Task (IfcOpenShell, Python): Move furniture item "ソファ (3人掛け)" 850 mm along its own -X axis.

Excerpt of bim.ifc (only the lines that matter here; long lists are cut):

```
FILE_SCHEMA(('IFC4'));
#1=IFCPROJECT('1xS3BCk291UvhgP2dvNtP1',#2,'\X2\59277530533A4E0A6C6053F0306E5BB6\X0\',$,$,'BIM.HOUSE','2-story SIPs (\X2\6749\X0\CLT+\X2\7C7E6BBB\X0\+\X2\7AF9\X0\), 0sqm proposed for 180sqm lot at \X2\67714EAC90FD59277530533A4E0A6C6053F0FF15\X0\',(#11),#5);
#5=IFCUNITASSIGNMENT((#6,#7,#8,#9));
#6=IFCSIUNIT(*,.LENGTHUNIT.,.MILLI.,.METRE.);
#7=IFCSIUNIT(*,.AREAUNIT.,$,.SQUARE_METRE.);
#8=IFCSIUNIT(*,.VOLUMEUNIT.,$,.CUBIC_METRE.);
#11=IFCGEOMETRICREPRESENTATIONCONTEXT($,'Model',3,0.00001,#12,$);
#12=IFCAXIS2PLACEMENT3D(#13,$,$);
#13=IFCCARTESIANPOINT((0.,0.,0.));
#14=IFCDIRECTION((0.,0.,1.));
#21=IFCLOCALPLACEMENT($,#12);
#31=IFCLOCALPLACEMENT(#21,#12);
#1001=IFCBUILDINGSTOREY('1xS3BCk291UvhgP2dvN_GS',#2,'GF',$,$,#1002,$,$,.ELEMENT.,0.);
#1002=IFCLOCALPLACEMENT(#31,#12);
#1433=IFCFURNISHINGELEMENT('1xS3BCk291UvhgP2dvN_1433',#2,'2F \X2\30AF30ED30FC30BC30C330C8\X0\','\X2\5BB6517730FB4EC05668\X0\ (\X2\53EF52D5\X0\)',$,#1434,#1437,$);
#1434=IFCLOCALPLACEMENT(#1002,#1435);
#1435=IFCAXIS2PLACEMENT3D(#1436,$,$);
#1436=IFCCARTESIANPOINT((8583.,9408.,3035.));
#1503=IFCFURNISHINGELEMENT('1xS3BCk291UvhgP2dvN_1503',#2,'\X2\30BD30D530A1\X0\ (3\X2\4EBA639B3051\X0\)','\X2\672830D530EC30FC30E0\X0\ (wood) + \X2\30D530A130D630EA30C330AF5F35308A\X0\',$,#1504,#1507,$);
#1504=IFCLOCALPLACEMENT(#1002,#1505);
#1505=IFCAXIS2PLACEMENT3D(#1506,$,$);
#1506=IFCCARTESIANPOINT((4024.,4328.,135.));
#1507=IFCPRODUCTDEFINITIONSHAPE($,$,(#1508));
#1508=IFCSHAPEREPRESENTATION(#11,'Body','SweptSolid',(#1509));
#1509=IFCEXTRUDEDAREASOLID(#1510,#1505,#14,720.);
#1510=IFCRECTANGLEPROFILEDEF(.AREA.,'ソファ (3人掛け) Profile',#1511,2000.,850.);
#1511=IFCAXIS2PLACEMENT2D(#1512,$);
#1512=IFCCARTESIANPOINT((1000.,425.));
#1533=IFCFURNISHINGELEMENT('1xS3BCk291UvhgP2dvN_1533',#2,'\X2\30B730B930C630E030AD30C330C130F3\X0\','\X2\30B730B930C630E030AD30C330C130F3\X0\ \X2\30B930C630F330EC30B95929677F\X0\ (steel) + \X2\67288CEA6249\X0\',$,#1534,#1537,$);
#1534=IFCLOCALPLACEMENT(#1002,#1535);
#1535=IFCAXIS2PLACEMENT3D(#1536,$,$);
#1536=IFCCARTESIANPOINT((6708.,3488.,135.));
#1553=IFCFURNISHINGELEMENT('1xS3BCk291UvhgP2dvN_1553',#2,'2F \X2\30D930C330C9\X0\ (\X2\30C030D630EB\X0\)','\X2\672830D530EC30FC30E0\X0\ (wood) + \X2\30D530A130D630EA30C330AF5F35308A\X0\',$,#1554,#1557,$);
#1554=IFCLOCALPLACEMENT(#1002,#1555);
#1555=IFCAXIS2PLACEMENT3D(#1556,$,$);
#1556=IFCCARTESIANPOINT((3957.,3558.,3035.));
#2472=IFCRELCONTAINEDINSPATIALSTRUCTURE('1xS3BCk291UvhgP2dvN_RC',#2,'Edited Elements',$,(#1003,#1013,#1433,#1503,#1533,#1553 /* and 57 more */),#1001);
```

```python
import ifcopenshell
import ifcopenshell.api.geometry
import ifcopenshell.util.placement
import ifcopenshell.util.unit

model = ifcopenshell.open("bim.ifc")
unit_scale = ifcopenshell.util.unit.calculate_unit_scale(model)

item = model.by_guid("1xS3BCk291UvhgP2dvN_1503")
matrix = ifcopenshell.util.placement.get_local_placement(item.ObjectPlacement)
matrix[:3, 3] -= matrix[:3, 0] * 0.85 / unit_scale
ifcopenshell.api.geometry.edit_object_placement(model, product=item, matrix=matrix, is_si=False)

print(ifcopenshell.util.placement.get_local_placement(item.ObjectPlacement).round(3) + 0.0)

model.write("bim_v2.ifc")
```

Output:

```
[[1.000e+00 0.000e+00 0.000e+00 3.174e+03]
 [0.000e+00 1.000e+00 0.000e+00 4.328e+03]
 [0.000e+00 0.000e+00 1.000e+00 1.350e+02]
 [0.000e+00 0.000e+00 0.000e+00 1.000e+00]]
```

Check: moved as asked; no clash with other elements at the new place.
